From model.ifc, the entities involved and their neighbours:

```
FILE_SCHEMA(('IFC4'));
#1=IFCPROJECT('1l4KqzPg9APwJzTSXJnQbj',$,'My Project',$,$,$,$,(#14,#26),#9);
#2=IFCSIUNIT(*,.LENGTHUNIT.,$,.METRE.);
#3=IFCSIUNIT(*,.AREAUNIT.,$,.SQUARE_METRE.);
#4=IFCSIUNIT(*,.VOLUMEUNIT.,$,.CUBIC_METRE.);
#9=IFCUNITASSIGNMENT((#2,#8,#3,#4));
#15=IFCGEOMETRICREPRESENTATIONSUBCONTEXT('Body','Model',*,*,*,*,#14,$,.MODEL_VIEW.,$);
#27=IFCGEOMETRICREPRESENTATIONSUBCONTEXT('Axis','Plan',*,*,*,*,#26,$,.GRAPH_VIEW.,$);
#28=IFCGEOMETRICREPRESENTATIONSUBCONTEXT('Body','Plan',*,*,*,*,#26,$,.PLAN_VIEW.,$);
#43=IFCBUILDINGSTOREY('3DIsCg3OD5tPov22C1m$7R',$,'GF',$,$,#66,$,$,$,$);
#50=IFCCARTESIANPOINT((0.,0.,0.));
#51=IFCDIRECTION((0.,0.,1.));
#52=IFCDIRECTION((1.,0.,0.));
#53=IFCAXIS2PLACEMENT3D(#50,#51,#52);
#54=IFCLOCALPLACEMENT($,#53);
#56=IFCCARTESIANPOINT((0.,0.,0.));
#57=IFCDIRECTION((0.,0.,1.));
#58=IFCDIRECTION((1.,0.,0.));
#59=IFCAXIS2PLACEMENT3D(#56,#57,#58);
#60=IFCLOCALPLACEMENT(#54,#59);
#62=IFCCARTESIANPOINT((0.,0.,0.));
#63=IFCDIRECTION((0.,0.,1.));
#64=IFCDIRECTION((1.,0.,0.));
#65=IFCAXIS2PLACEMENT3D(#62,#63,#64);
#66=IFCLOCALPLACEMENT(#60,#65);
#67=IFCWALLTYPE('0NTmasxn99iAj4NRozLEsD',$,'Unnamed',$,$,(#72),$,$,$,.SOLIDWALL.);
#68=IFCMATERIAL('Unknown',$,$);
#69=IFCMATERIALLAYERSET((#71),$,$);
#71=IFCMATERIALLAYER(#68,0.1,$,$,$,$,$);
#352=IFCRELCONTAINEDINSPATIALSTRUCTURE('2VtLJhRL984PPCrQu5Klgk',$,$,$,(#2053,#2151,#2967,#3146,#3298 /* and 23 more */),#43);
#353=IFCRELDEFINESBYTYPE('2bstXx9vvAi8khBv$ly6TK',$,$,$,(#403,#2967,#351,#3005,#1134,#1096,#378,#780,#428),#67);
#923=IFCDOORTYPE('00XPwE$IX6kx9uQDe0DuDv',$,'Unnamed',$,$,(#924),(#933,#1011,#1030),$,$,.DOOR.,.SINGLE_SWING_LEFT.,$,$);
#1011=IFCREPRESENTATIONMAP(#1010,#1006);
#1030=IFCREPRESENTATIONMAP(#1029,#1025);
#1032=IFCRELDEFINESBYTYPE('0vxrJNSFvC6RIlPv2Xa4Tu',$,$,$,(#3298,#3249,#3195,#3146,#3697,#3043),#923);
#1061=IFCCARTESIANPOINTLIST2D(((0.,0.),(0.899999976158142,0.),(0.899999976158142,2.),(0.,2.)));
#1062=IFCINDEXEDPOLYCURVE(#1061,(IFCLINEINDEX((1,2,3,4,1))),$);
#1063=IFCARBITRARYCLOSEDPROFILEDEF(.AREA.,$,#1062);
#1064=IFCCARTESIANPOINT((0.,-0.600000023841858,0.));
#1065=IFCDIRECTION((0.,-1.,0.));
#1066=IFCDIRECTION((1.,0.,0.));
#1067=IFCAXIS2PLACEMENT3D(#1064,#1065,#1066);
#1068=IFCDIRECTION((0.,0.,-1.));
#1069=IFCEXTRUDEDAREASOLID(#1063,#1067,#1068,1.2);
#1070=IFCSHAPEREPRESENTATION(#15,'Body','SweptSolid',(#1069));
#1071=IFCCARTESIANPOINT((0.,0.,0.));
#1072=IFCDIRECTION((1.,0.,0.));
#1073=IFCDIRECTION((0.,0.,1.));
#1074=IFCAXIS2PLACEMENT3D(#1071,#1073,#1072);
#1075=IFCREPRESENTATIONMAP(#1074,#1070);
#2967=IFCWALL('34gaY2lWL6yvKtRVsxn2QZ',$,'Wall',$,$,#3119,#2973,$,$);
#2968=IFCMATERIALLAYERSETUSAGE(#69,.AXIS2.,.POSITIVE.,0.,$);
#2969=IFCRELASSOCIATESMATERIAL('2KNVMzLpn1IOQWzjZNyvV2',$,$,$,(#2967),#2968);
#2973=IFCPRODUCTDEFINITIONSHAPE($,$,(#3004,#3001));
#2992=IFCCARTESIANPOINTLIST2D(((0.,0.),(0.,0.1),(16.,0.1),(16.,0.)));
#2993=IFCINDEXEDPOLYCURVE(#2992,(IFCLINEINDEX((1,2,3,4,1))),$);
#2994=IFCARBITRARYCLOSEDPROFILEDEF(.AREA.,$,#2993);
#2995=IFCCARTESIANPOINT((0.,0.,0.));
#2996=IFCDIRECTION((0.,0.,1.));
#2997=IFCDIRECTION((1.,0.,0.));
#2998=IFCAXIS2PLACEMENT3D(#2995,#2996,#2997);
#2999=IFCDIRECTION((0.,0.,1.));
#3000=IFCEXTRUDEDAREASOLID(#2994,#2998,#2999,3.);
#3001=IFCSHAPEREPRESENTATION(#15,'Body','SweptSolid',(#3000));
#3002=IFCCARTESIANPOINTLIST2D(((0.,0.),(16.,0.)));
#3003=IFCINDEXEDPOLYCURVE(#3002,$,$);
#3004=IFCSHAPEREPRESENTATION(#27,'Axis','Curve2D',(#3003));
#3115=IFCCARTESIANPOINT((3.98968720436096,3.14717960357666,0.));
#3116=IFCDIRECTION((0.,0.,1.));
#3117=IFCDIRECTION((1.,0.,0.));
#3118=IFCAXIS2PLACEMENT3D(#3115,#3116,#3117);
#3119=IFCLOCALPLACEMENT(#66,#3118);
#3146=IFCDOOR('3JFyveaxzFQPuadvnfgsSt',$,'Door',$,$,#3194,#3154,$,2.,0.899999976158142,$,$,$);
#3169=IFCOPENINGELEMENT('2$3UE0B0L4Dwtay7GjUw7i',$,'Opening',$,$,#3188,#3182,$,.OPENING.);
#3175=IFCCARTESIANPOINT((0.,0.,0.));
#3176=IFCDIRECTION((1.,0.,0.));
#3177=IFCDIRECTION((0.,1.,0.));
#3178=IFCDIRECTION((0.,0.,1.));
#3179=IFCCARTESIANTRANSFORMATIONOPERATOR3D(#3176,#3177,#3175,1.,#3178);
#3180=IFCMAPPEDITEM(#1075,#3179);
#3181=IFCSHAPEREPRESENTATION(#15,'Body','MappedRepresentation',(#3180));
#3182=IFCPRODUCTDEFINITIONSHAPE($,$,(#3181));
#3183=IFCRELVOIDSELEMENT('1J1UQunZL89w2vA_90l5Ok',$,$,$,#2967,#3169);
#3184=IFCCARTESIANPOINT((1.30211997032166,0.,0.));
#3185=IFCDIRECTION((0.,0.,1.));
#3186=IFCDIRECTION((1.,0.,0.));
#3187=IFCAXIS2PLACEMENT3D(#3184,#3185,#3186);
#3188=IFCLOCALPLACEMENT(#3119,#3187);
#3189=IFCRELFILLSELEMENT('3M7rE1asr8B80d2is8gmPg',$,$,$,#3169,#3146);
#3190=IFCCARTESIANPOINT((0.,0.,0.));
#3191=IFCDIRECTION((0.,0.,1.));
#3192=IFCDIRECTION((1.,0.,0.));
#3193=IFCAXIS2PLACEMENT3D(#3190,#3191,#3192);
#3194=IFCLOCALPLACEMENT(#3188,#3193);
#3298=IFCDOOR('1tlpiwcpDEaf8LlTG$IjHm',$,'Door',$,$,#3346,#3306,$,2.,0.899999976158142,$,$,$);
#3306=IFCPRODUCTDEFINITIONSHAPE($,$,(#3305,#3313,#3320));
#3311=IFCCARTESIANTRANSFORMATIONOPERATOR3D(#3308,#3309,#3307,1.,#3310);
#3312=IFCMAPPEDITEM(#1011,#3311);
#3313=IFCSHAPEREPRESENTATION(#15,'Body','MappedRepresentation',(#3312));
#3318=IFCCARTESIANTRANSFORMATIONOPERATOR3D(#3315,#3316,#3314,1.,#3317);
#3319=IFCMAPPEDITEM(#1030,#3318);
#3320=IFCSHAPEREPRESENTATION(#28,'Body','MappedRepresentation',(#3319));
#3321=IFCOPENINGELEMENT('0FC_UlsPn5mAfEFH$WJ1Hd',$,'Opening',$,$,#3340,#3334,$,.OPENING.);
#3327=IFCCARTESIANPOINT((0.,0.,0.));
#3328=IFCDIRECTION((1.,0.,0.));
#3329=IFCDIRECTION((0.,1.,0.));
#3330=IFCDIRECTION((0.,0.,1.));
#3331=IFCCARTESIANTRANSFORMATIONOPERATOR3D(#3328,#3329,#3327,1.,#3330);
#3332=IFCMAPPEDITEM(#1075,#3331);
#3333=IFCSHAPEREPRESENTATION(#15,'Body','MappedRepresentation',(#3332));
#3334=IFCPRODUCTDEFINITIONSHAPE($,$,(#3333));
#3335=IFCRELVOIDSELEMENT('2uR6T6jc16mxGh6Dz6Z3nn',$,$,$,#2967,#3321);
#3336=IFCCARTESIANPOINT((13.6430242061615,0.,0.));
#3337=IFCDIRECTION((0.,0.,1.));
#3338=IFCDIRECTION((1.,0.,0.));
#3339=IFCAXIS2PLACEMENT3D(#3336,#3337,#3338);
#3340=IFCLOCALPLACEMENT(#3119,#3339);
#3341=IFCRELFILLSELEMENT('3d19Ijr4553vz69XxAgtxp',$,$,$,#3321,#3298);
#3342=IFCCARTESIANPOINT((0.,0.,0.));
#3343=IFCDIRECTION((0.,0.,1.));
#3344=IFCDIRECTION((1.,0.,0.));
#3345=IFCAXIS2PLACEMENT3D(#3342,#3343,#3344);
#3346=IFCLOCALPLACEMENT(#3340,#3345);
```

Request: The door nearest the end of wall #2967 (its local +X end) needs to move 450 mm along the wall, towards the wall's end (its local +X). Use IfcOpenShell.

```python
import ifcopenshell
import ifcopenshell.api.geometry
import ifcopenshell.util.placement

model = ifcopenshell.open("model.ifc")

door = model.by_id(3298)
opening = door.FillsVoids[0].RelatingOpeningElement
wall = opening.VoidsElements[0].RelatingBuildingElement

wall_matrix = ifcopenshell.util.placement.get_local_placement(wall.ObjectPlacement)
shift = wall_matrix[:3, 0] * 0.45
before = ifcopenshell.util.placement.get_local_placement(door.ObjectPlacement)[:3, 3].copy()

# The door is placed relative to its opening, so it follows when the opening moves.
matrix = ifcopenshell.util.placement.get_local_placement(opening.ObjectPlacement)
matrix[:3, 3] += shift
ifcopenshell.api.geometry.edit_object_placement(
    model, product=opening, matrix=matrix, is_si=False, should_transform_children=True
)

after = ifcopenshell.util.placement.get_local_placement(door.ObjectPlacement)[:3, 3]
print("door moved by", (after - before).round(3) + 0.0)

model.write("model-out.ifc")
```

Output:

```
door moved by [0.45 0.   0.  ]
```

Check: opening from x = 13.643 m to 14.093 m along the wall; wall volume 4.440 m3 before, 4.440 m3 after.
